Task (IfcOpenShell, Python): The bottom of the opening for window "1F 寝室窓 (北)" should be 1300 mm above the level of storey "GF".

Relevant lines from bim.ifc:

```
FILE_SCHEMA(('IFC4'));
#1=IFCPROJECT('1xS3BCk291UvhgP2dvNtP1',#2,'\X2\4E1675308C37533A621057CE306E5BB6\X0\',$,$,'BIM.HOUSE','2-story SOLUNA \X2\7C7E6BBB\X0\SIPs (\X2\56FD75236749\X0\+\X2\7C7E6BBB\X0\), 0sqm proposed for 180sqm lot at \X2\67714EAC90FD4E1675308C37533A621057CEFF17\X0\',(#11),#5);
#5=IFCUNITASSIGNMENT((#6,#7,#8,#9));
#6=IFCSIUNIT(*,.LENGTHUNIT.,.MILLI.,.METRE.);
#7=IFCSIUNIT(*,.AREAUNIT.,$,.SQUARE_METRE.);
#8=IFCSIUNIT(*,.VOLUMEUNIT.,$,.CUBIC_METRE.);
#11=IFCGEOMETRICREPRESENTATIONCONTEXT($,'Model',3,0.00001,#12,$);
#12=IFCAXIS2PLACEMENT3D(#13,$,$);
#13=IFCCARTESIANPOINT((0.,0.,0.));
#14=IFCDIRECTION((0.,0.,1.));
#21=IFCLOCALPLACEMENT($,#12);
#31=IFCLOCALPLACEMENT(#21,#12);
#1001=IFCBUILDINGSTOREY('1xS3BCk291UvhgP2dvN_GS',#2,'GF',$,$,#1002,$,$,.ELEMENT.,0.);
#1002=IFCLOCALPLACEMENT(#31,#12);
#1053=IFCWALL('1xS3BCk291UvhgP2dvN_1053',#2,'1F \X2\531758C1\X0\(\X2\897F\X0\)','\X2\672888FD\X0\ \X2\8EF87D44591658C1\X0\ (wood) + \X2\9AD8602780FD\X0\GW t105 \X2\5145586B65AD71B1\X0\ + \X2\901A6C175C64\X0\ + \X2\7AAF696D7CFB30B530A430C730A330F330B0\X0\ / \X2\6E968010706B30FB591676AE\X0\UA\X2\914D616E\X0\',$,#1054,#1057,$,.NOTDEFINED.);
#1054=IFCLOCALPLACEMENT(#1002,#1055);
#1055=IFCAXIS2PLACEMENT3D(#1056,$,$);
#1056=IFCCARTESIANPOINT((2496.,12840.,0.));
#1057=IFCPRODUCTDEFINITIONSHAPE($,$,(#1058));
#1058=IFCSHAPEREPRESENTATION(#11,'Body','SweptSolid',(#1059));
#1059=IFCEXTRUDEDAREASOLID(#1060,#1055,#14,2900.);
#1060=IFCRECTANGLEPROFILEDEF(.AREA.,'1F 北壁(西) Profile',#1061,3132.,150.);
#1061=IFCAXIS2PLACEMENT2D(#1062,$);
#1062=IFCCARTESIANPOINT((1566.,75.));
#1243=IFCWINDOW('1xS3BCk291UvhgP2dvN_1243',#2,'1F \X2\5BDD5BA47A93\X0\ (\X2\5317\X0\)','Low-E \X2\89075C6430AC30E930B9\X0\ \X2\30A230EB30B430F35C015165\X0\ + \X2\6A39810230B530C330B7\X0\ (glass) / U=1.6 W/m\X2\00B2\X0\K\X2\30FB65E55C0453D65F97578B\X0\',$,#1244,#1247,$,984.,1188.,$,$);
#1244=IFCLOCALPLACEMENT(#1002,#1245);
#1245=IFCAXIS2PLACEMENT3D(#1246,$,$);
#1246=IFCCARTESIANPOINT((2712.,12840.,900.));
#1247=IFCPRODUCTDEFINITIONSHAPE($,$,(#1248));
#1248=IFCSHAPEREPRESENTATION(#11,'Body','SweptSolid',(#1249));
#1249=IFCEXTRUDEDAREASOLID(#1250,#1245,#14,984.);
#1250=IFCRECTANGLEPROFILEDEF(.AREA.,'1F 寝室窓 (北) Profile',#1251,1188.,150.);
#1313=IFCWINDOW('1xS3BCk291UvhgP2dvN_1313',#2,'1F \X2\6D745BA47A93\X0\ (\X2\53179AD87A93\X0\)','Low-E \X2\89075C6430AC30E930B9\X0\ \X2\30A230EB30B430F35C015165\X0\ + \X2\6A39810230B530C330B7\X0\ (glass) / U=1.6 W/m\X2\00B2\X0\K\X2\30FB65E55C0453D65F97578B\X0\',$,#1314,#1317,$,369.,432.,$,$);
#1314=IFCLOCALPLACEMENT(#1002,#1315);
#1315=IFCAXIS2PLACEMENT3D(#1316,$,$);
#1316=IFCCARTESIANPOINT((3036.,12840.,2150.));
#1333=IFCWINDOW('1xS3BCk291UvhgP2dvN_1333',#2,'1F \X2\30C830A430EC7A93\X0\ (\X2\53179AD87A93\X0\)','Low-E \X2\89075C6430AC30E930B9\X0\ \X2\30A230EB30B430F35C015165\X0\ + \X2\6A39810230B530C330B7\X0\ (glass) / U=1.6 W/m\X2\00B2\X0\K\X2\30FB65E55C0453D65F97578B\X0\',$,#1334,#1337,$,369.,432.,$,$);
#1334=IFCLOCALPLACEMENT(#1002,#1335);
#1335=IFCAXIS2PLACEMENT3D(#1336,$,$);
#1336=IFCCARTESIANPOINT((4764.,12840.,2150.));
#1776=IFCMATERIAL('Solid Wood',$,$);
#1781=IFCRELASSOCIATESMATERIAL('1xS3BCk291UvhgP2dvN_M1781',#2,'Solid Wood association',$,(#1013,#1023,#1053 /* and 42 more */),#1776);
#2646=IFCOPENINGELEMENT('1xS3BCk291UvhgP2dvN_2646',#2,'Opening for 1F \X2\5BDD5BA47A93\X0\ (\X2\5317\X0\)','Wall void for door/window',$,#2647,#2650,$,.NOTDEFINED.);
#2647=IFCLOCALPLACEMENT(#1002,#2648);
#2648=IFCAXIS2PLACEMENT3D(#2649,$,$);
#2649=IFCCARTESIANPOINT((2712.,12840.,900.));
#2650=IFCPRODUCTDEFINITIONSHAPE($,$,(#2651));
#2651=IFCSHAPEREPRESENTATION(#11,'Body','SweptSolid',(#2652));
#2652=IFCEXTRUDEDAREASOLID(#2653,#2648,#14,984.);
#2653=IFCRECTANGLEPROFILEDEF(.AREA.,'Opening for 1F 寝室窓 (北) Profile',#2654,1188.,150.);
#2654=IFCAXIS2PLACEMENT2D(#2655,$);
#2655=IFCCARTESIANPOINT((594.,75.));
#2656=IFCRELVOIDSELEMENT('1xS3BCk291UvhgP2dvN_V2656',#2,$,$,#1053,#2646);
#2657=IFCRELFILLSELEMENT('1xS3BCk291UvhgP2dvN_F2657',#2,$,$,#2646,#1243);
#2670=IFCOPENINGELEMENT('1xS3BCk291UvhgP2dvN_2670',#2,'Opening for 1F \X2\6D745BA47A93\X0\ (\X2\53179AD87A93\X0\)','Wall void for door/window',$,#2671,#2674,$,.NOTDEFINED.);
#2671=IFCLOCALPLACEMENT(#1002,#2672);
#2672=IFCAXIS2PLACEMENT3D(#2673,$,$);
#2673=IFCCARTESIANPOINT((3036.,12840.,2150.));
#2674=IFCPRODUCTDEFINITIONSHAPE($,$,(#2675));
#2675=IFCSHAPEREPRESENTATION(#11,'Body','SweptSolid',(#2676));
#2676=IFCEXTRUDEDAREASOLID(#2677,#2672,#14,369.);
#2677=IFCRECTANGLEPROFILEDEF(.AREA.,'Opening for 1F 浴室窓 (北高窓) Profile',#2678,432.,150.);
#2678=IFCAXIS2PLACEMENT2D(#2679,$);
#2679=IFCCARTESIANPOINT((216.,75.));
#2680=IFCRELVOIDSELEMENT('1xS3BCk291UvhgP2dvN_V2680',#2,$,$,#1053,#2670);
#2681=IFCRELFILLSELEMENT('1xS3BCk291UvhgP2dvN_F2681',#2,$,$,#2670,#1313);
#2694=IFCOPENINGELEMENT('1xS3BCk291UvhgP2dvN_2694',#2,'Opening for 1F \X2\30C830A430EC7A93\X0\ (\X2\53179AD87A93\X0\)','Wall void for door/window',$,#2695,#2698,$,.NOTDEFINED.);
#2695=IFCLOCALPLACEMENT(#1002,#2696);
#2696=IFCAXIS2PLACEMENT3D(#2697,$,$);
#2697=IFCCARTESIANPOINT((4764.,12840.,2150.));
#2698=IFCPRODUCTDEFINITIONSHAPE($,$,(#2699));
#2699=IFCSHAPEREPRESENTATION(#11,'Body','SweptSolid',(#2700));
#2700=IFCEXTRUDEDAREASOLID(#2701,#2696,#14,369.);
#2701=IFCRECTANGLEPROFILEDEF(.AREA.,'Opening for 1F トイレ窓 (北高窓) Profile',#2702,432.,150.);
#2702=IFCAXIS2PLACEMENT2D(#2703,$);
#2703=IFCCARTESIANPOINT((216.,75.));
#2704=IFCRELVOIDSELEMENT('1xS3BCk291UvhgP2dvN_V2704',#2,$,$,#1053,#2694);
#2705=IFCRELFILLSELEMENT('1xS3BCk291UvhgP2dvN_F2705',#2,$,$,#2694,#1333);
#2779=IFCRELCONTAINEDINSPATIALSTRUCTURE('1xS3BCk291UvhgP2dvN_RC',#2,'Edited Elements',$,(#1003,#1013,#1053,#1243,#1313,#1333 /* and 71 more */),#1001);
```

```python
import numpy as np
import ifcopenshell
import ifcopenshell.api.geometry
import ifcopenshell.geom
import ifcopenshell.util.element
import ifcopenshell.util.placement
import ifcopenshell.util.shape
import ifcopenshell.util.unit

model = ifcopenshell.open("bim.ifc")
unit_scale = ifcopenshell.util.unit.calculate_unit_scale(model)

window = model.by_guid("1xS3BCk291UvhgP2dvN_1243")
opening = window.FillsVoids[0].RelatingOpeningElement
storey = ifcopenshell.util.element.get_container(window, ifc_class="IfcBuildingStorey")
level = ifcopenshell.util.placement.get_local_placement(storey.ObjectPlacement)[2, 3]

# The opening's origin need not be at the sill, so measure its lowest point.
shape = ifcopenshell.geom.create_shape(ifcopenshell.geom.settings(), opening)
bottom = ifcopenshell.util.shape.get_shape_bottom_elevation(shape, shape.geometry) / unit_scale
dz = level + 1300.0 - bottom

shift = np.array([0.0, 0.0, dz])
# The window is not placed relative to its opening, so move both.
for product in (opening, window):
    matrix = ifcopenshell.util.placement.get_local_placement(product.ObjectPlacement)
    matrix[:3, 3] += shift
    ifcopenshell.api.geometry.edit_object_placement(model, product=product, matrix=matrix, is_si=False)

print(f"moved by {dz * unit_scale:+.3f} m")

model.write("bim_rev.ifc")
```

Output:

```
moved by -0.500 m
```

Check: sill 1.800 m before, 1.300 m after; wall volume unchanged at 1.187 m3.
